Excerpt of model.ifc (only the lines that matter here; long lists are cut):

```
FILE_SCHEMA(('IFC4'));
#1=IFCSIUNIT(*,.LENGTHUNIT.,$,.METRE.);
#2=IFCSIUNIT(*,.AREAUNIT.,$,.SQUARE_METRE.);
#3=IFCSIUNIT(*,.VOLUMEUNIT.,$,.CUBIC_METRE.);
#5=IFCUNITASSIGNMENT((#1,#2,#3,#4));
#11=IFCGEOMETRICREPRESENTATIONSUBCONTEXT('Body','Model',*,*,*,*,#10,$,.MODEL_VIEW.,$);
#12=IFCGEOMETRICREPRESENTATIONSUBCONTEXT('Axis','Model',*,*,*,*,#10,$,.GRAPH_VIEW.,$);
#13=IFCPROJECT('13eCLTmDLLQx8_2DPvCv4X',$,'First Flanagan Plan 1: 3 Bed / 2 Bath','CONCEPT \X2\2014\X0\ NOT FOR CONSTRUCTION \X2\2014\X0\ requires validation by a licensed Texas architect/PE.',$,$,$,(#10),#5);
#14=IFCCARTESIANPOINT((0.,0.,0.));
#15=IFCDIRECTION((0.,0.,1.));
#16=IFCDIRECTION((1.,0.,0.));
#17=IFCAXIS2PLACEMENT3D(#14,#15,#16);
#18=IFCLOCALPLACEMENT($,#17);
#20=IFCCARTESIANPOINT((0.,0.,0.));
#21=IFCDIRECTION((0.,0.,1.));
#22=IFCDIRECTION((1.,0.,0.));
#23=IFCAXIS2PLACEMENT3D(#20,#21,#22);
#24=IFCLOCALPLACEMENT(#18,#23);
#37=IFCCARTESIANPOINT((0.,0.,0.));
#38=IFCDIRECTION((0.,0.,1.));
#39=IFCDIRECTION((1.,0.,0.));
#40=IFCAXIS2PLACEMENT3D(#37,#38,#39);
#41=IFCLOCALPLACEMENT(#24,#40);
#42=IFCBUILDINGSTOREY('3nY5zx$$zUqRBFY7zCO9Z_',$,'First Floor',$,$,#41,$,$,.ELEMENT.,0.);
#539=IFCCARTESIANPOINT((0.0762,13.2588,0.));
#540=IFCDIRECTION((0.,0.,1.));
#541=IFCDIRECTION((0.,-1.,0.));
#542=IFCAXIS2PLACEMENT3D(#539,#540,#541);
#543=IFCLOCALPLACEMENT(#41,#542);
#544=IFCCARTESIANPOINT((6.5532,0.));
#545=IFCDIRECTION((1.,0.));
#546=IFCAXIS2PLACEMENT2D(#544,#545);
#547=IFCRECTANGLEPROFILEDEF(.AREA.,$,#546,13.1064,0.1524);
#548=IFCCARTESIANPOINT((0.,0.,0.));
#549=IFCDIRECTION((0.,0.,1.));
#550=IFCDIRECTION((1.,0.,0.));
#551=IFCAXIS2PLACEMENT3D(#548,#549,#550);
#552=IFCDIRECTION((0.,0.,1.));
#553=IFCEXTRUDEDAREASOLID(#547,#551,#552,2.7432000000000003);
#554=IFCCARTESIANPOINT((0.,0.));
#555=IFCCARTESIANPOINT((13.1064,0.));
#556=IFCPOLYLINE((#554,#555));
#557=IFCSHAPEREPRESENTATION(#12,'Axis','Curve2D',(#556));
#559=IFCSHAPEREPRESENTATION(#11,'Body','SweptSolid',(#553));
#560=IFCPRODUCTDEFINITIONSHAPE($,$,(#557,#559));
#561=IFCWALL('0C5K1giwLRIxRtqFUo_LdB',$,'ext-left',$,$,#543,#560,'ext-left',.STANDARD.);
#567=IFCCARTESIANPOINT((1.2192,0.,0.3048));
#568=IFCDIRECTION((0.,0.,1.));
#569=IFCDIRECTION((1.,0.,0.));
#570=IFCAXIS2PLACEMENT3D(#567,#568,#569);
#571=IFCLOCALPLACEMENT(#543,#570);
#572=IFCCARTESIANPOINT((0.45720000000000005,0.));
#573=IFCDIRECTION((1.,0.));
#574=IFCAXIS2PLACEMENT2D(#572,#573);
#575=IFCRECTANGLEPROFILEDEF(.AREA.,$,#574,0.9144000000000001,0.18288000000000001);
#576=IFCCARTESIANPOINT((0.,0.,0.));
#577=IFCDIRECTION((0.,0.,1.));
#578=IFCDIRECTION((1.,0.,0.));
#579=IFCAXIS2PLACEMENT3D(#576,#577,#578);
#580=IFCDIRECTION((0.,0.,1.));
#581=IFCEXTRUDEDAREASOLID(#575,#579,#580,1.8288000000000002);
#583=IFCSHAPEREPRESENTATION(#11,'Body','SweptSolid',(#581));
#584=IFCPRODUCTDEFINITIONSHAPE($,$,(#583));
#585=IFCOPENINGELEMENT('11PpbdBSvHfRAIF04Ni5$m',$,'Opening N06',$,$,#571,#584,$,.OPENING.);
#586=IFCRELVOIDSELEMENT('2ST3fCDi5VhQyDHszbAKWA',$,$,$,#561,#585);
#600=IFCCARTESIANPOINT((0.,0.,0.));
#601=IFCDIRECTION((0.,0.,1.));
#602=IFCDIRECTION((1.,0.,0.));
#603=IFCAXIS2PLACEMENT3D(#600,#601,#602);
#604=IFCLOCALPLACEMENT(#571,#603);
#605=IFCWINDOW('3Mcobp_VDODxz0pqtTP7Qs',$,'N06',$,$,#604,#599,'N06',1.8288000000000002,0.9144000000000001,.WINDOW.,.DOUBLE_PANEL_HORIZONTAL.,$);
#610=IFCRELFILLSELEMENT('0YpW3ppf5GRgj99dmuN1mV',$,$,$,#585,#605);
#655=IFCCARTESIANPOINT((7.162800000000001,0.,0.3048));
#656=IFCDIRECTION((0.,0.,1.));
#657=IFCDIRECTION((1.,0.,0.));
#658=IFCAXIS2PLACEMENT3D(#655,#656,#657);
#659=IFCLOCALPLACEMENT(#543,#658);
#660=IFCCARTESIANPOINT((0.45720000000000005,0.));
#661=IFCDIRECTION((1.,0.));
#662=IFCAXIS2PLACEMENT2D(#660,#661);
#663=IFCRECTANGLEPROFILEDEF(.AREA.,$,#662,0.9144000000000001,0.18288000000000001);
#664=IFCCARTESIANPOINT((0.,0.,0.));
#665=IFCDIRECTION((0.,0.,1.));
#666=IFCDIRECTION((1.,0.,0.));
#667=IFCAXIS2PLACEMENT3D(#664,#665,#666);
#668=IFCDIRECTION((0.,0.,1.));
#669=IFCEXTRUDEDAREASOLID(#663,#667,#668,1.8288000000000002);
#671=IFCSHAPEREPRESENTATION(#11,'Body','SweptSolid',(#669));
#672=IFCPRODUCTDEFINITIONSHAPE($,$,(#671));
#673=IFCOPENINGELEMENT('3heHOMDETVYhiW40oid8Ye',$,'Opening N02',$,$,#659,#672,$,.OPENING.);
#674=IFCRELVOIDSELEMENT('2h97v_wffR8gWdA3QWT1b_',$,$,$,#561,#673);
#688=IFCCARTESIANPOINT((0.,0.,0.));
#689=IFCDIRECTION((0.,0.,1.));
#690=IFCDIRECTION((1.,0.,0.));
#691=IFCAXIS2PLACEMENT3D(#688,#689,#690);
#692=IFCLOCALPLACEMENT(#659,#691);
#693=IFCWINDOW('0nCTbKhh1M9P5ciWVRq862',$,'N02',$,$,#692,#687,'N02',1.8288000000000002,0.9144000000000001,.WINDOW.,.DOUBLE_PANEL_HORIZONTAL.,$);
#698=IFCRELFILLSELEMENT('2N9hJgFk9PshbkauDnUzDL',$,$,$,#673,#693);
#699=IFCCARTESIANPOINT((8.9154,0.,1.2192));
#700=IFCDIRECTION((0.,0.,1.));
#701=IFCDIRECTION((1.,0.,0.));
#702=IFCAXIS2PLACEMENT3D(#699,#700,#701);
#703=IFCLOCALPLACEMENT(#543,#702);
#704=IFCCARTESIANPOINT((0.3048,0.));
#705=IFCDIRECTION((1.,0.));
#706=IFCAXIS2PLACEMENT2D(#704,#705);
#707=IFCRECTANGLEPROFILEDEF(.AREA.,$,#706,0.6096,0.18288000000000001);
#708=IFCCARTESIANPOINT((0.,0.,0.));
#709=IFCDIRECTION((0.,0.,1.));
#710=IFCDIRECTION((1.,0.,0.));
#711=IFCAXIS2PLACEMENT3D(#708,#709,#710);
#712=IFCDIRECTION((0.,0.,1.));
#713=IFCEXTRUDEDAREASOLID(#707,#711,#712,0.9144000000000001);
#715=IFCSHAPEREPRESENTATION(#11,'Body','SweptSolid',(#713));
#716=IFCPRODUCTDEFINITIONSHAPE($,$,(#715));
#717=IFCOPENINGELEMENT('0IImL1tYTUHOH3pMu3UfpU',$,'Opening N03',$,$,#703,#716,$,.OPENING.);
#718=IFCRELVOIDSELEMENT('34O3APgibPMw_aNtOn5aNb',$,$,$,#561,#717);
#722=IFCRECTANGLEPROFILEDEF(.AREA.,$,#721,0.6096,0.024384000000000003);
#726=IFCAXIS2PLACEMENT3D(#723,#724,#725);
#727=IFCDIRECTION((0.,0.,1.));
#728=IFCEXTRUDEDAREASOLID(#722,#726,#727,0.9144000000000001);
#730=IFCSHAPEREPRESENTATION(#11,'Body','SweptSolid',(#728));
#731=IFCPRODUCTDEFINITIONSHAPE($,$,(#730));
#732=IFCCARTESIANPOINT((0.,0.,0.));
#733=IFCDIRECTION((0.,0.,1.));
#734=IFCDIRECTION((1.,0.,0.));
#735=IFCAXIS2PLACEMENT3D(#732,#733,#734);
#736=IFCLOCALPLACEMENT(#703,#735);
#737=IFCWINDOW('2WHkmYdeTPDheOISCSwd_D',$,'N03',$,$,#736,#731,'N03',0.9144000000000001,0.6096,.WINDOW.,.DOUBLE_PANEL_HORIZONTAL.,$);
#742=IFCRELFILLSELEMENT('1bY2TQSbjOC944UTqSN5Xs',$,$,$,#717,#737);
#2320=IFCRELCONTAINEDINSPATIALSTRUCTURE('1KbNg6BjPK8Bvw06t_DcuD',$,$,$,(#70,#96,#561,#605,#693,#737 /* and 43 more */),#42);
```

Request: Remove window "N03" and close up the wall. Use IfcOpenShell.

```python
import ifcopenshell
import ifcopenshell.api.feature
import ifcopenshell.api.root
import ifcopenshell.geom
import ifcopenshell.util.shape

model = ifcopenshell.open("model.ifc")
settings = ifcopenshell.geom.settings()


def volume(element):
    """Net volume in cubic metres, openings subtracted."""
    shape = ifcopenshell.geom.create_shape(settings, element)
    return ifcopenshell.util.shape.get_volume(shape.geometry)


window = model.by_id(737)
opening = window.FillsVoids[0].RelatingOpeningElement
wall = opening.VoidsElements[0].RelatingBuildingElement
before = volume(wall)

ifcopenshell.api.root.remove_product(model, product=window)
ifcopenshell.api.feature.remove_feature(model, feature=opening)

after = volume(wall)

print(f"wall volume {before:.3f} -> {after:.3f} m3")

model.write("model-out.ifc")
```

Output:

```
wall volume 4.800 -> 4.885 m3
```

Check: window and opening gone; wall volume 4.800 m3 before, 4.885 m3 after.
